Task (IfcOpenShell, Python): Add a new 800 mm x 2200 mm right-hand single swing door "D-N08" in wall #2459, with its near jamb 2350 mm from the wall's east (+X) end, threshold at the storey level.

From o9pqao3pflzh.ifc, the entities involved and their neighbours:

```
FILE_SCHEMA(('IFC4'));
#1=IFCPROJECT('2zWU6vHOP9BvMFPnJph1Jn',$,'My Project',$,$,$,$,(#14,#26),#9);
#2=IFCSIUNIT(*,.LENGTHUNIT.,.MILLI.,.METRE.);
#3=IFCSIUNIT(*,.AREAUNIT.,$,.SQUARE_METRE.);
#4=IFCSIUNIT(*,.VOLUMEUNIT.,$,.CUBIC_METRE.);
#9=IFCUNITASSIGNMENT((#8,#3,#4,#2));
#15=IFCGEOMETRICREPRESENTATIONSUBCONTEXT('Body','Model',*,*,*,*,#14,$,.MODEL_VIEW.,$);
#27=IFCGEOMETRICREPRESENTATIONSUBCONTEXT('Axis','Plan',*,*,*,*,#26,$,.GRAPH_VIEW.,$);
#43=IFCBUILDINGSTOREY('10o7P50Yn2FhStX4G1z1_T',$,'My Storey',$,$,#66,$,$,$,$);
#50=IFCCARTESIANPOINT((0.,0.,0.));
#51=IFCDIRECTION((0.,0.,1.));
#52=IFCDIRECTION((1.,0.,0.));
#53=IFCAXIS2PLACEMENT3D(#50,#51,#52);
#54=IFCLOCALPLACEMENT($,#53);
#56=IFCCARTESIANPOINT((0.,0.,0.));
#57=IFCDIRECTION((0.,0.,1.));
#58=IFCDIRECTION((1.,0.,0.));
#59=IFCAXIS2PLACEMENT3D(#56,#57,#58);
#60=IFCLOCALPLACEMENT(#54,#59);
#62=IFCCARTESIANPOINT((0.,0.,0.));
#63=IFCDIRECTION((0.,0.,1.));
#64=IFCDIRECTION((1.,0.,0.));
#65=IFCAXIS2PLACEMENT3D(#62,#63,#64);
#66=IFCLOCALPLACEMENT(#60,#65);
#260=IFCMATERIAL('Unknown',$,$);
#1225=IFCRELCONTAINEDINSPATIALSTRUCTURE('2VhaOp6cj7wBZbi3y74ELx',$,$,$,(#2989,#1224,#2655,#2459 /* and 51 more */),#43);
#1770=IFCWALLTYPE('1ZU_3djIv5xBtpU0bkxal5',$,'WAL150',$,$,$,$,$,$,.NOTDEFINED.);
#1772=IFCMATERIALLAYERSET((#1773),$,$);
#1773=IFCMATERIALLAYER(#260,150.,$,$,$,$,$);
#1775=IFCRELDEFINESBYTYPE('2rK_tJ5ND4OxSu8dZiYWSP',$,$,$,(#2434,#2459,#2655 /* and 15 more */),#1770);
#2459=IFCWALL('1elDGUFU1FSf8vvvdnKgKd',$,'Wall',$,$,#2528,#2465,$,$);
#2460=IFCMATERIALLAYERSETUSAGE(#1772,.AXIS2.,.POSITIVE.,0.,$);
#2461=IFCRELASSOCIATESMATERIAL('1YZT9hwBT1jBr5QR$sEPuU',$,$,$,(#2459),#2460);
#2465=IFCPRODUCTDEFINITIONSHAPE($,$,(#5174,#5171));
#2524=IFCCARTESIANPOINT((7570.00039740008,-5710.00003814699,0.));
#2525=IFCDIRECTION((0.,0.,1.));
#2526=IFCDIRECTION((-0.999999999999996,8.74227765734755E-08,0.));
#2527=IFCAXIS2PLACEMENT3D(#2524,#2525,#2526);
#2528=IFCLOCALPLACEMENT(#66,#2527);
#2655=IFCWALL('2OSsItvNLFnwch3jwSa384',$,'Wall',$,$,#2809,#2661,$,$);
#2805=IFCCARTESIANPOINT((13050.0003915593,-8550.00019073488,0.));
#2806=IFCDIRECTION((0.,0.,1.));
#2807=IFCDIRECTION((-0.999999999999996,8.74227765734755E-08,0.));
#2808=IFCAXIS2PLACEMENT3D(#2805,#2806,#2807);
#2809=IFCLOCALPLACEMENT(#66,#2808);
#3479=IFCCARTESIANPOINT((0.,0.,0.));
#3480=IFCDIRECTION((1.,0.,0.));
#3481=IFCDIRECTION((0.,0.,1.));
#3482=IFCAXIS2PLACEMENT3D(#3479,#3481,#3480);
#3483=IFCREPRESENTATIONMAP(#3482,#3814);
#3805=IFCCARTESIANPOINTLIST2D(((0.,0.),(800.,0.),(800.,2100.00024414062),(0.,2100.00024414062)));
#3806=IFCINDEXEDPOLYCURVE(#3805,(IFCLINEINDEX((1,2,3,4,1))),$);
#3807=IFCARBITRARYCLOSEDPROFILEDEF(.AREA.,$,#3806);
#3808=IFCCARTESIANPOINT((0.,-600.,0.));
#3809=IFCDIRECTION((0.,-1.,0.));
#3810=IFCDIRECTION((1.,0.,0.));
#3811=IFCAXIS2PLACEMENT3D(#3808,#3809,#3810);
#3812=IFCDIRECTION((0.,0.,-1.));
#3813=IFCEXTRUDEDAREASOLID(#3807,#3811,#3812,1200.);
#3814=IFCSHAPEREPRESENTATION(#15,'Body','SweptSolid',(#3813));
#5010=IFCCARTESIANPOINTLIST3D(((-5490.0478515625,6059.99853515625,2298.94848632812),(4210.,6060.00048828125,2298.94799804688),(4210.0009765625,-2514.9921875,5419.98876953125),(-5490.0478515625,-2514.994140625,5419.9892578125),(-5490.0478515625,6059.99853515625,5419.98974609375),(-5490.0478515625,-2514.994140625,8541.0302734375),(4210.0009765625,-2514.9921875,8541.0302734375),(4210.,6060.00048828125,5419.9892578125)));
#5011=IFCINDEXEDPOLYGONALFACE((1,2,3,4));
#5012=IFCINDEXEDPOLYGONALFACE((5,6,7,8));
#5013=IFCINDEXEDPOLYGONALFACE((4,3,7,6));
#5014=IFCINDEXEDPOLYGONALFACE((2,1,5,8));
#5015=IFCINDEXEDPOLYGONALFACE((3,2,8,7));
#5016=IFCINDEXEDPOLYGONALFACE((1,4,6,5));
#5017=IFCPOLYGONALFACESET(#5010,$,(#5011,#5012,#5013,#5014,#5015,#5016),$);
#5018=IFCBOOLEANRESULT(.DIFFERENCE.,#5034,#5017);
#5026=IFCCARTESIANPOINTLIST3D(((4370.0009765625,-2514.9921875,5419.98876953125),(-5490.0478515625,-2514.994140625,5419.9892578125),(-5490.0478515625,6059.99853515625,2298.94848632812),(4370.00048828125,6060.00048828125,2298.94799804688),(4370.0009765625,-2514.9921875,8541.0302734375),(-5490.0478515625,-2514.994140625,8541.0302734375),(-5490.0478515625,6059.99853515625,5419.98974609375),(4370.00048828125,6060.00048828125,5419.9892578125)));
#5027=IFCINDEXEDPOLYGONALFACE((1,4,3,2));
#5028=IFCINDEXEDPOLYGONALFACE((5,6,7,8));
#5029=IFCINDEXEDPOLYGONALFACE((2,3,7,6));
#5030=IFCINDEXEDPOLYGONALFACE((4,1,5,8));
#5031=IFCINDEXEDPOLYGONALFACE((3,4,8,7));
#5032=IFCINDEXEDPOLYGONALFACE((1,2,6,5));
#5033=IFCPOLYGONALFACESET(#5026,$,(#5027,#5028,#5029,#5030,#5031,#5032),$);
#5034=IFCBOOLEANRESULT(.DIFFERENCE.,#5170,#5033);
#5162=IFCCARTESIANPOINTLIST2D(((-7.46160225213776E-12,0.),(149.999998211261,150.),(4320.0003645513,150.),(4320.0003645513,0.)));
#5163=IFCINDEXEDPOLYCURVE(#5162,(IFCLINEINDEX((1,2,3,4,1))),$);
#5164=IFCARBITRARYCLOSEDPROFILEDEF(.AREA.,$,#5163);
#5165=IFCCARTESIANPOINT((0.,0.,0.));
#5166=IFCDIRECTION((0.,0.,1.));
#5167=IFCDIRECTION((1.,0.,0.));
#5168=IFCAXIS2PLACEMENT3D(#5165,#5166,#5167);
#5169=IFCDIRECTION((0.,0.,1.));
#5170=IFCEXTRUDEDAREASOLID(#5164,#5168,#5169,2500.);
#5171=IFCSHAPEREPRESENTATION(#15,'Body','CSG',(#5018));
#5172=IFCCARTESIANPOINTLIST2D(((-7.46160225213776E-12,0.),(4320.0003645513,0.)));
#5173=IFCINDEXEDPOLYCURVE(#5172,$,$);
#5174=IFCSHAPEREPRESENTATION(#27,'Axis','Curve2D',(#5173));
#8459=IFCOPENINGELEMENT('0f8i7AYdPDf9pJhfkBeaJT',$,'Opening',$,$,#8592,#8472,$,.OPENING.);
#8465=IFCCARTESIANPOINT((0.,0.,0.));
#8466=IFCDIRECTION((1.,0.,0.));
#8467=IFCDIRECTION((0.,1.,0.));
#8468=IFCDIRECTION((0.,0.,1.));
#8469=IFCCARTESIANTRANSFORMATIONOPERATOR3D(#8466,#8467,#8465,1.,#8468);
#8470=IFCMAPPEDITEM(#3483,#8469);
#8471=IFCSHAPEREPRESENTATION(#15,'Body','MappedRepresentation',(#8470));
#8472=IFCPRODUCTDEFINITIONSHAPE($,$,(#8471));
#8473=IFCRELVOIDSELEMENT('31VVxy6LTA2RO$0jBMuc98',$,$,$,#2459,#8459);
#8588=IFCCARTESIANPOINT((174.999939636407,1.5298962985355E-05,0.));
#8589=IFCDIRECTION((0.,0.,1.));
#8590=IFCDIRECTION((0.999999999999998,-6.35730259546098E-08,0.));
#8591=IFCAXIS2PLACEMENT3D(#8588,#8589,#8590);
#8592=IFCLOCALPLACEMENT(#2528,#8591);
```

```python
import numpy as np
import ifcopenshell
import ifcopenshell.api.feature
import ifcopenshell.api.geometry
import ifcopenshell.api.root
import ifcopenshell.api.spatial
import ifcopenshell.geom
import ifcopenshell.util.element
import ifcopenshell.util.placement
import ifcopenshell.util.representation
import ifcopenshell.util.shape
import ifcopenshell.util.unit

model = ifcopenshell.open("o9pqao3pflzh.ifc")
unit_scale = ifcopenshell.util.unit.calculate_unit_scale(model)
settings = ifcopenshell.geom.settings()


def volume(element):
    """Net volume in cubic metres, openings subtracted."""
    shape = ifcopenshell.geom.create_shape(settings, element)
    return ifcopenshell.util.shape.get_volume(shape.geometry)


wall = model.by_guid("1elDGUFU1FSf8vvvdnKgKd")
storey = ifcopenshell.util.element.get_container(wall, ifc_class="IfcBuildingStorey")
context = ifcopenshell.util.representation.get_context(model, "Model", "Body", "MODEL_VIEW")
before = volume(wall)

width, height, from_end, sill = 0.8, 2.2, 2.35, 0.0  # metres

# The wall runs along its own X axis, and the end named is its -X end.
wall_shape = ifcopenshell.geom.create_shape(settings, wall)
x, y, z = ifcopenshell.util.shape.get_vertices(wall_shape.geometry).T
start = x.min() + from_end
face, thickness = float(y.min()), float(y.max() - y.min())
wall_matrix = ifcopenshell.util.placement.get_local_placement(wall.ObjectPlacement)
level = ifcopenshell.util.placement.get_local_placement(storey.ObjectPlacement)[2, 3]


def in_wall(x, y):
    """Placement at x, y metres in the wall's axes, at sill height."""
    matrix = wall_matrix.copy()
    matrix[:, 3] = wall_matrix @ np.array([x / unit_scale, y / unit_scale, 0.0, 1.0])
    matrix[2, 3] = level + sill / unit_scale
    return matrix


# Opening: a box that overshoots both wall faces by 50 mm.
opening = ifcopenshell.api.root.create_entity(model, ifc_class="IfcOpeningElement", predefined_type="OPENING")
box = ifcopenshell.api.geometry.add_wall_representation(
    model, context=context, length=width, height=height, thickness=thickness + 0.1
)
ifcopenshell.api.geometry.assign_representation(model, product=opening, representation=box)
ifcopenshell.api.geometry.edit_object_placement(model, product=opening, matrix=in_wall(start, face - 0.05), is_si=False)
ifcopenshell.api.feature.add_feature(model, feature=opening, element=wall)

door = ifcopenshell.api.root.create_entity(model, ifc_class="IfcDoor", name="D-N08", predefined_type="DOOR")
door.OverallWidth, door.OverallHeight = width / unit_scale, height / unit_scale
door.OperationType = "SINGLE_SWING_RIGHT"
body = ifcopenshell.api.geometry.add_door_representation(
    model,
    context=context,
    overall_width=door.OverallWidth,
    overall_height=door.OverallHeight,
    operation_type="SINGLE_SWING_RIGHT",
    lining_properties={"LiningDepth": thickness / unit_scale, "ThresholdDepth": thickness / unit_scale},
)
ifcopenshell.api.geometry.assign_representation(model, product=door, representation=body)
ifcopenshell.api.spatial.assign_container(model, products=[door], relating_structure=storey)
ifcopenshell.api.feature.add_filling(model, opening=opening, element=door)

# The lining spans the wall, so the door starts at the wall face.
ifcopenshell.api.geometry.edit_object_placement(model, product=door, matrix=in_wall(start, face), is_si=False)

after = volume(wall)

print(f"wall volume {before:.3f} -> {after:.3f} m3")

model.write("o9pqao3pflzh_v2.ifc")
```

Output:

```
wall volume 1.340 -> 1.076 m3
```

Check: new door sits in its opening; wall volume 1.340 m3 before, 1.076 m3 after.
